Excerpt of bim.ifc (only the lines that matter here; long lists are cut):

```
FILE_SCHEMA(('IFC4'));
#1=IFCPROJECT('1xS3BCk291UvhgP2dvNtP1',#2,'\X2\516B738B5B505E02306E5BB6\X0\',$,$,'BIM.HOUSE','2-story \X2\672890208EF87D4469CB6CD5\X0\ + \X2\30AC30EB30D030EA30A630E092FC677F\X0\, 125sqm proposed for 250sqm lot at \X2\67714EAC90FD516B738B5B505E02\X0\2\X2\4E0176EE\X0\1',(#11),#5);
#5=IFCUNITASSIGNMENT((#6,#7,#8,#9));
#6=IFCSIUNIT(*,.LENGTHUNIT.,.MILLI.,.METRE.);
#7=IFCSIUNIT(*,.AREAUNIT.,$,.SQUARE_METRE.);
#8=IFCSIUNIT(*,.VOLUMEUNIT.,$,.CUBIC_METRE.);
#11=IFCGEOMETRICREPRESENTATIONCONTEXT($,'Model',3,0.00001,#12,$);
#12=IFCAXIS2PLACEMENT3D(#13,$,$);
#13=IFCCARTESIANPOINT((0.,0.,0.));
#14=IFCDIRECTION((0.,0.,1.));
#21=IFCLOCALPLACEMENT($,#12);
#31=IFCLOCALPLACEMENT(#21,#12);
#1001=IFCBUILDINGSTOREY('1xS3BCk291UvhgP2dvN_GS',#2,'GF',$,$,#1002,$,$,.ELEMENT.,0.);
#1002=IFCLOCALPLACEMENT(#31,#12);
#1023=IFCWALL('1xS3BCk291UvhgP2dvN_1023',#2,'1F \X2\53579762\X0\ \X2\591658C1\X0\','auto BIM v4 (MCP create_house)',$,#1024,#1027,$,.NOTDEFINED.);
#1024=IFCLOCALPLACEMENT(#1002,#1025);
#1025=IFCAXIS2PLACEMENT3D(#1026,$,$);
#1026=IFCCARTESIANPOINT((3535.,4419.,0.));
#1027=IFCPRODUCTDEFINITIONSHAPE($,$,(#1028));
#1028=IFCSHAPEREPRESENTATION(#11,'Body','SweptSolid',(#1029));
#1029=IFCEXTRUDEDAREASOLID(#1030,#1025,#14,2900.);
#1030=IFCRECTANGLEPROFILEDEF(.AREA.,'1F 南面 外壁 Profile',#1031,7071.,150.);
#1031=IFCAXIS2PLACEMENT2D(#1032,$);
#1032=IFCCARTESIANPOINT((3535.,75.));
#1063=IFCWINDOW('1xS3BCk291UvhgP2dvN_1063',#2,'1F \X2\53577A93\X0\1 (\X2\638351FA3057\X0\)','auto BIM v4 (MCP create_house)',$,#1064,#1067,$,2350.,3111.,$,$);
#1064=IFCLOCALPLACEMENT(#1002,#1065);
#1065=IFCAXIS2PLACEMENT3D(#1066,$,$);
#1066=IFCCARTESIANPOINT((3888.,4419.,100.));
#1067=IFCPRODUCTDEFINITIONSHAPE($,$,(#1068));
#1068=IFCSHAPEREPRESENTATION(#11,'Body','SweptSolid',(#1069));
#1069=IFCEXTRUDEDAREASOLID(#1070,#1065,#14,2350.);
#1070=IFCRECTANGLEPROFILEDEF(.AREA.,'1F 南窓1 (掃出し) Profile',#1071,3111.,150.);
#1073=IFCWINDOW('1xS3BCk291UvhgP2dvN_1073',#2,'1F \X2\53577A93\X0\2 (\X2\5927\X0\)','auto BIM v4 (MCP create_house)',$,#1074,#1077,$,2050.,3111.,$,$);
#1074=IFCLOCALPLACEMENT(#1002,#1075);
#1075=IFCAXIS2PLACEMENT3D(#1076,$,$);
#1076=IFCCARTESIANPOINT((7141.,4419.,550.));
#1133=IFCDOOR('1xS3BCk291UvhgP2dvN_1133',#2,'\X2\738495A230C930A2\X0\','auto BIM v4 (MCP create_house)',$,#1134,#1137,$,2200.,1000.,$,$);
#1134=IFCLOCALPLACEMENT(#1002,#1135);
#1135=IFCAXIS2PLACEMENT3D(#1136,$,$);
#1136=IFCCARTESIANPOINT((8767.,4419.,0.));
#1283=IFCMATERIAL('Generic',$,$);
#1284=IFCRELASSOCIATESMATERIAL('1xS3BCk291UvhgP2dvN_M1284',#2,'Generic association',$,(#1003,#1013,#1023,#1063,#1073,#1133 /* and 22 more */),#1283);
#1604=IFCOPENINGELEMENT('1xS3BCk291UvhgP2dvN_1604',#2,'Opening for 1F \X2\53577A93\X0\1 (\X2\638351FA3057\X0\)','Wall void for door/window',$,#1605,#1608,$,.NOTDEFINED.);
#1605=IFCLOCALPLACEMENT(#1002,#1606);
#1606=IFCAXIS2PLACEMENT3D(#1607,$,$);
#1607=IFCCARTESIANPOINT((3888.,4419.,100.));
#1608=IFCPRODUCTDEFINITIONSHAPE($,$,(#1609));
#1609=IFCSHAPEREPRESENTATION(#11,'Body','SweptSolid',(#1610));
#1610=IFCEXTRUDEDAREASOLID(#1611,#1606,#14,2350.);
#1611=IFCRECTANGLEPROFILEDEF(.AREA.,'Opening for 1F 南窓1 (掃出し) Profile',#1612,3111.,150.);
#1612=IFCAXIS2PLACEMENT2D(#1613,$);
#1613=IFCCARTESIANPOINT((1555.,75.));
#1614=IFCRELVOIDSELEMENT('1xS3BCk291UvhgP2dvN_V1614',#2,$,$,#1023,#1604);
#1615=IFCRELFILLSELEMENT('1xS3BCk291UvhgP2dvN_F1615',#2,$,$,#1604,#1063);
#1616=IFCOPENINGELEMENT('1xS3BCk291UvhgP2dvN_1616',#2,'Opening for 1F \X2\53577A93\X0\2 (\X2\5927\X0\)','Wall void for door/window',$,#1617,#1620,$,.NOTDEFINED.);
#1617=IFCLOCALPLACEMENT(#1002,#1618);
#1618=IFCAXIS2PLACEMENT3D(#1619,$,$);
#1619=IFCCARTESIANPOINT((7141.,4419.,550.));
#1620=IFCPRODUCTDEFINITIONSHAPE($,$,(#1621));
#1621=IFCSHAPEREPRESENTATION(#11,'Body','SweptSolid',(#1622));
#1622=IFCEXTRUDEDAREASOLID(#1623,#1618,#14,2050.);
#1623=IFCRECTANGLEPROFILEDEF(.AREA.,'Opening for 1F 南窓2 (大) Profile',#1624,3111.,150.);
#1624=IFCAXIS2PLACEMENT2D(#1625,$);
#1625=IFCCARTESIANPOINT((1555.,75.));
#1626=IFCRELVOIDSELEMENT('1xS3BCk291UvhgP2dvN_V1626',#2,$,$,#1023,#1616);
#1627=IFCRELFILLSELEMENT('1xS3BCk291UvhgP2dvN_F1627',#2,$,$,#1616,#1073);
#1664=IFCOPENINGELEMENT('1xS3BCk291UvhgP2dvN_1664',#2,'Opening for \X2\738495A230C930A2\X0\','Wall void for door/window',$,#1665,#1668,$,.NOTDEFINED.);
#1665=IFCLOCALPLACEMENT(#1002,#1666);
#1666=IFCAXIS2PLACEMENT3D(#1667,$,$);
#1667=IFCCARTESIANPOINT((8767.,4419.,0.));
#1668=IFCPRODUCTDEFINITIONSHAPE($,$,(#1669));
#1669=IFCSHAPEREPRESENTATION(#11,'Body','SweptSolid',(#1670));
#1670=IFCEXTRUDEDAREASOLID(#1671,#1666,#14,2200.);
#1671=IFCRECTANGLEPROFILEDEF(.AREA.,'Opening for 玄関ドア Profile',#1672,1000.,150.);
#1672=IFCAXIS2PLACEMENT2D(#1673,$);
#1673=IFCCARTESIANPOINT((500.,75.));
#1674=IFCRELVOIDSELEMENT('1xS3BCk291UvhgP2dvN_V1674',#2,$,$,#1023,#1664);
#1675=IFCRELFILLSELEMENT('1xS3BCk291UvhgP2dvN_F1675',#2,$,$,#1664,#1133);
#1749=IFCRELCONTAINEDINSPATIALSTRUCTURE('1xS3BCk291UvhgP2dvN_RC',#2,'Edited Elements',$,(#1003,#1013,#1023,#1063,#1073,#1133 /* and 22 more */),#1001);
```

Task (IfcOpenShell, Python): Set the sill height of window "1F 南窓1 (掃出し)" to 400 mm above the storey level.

```python
import numpy as np
import ifcopenshell
import ifcopenshell.api.geometry
import ifcopenshell.geom
import ifcopenshell.util.element
import ifcopenshell.util.placement
import ifcopenshell.util.shape
import ifcopenshell.util.unit

model = ifcopenshell.open("bim.ifc")
unit_scale = ifcopenshell.util.unit.calculate_unit_scale(model)

window = model.by_guid("1xS3BCk291UvhgP2dvN_1063")
opening = window.FillsVoids[0].RelatingOpeningElement
storey = ifcopenshell.util.element.get_container(window, ifc_class="IfcBuildingStorey")
level = ifcopenshell.util.placement.get_local_placement(storey.ObjectPlacement)[2, 3]

# The opening's origin need not be at the sill, so measure its lowest point.
shape = ifcopenshell.geom.create_shape(ifcopenshell.geom.settings(), opening)
bottom = ifcopenshell.util.shape.get_shape_bottom_elevation(shape, shape.geometry) / unit_scale
dz = level + 400.0 - bottom

shift = np.array([0.0, 0.0, dz])
# The window is not placed relative to its opening, so move both.
for product in (opening, window):
    matrix = ifcopenshell.util.placement.get_local_placement(product.ObjectPlacement)
    matrix[:3, 3] += shift
    ifcopenshell.api.geometry.edit_object_placement(model, product=product, matrix=matrix, is_si=False)

print(f"moved by {dz * unit_scale:+.3f} m")

model.write("bim_updated.ifc")
```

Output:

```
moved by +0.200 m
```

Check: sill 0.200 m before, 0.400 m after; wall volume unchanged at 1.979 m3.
